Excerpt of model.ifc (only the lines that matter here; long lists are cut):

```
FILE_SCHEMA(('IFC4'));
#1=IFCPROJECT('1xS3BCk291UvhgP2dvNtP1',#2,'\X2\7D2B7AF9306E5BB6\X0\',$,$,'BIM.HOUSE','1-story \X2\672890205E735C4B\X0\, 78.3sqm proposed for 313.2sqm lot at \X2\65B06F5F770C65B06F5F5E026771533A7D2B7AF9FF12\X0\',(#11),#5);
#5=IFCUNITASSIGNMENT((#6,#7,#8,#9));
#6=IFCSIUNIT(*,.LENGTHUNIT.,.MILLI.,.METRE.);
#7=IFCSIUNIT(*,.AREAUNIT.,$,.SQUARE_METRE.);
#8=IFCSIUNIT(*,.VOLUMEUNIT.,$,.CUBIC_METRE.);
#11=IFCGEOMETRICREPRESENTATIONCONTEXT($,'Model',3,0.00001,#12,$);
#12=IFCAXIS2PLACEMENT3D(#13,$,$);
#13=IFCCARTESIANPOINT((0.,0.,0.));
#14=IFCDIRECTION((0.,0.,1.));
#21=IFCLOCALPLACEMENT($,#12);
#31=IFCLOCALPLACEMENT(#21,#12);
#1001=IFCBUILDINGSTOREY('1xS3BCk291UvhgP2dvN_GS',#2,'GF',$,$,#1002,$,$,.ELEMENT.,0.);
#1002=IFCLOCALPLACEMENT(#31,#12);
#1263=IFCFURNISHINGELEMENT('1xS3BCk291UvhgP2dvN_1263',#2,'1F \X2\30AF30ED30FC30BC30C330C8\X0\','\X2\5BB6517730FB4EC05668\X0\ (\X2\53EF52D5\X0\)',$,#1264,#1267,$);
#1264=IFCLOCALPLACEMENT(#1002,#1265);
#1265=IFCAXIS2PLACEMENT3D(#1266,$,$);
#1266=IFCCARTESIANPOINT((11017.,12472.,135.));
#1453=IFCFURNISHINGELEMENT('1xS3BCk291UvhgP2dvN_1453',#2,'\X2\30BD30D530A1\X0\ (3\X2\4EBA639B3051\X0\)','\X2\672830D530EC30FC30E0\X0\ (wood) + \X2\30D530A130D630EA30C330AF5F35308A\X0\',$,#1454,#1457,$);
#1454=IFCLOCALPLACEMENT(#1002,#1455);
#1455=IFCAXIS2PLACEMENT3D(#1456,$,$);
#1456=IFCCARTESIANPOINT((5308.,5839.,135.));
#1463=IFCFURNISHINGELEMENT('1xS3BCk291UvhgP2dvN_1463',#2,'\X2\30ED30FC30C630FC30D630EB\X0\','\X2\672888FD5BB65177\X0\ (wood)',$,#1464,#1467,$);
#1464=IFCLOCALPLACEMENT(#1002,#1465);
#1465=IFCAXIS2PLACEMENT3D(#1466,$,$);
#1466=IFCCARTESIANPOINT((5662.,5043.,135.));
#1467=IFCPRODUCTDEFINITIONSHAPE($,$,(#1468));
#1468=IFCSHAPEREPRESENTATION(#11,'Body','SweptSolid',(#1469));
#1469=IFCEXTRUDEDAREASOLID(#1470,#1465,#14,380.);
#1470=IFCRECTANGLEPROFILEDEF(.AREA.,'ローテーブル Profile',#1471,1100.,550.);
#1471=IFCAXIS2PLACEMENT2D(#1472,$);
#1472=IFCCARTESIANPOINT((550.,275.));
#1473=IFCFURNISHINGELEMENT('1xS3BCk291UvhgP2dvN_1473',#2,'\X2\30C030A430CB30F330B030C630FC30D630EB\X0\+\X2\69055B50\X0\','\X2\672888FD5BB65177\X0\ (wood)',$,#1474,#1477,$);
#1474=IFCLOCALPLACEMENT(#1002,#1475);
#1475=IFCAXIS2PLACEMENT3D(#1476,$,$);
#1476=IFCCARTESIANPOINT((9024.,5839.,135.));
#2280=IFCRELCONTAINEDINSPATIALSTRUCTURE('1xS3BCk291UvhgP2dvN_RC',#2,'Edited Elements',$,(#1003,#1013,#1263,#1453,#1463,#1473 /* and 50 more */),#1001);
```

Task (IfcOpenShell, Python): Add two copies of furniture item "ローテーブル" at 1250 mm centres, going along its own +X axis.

```python
import ifcopenshell
import ifcopenshell.api.geometry
import ifcopenshell.api.root
import ifcopenshell.util.element
import ifcopenshell.util.placement

model = ifcopenshell.open("model.ifc")


def reuse_history(source, copy):
    """copy_class also copies each property set's owner history, people and application; keep the originals."""
    for rel in copy.IsDefinedBy:
        if rel.is_a("IfcRelDefinesByProperties") and (history := rel.RelatingPropertyDefinition.OwnerHistory):
            rel.RelatingPropertyDefinition.OwnerHistory = source.OwnerHistory
            ifcopenshell.util.element.remove_deep2(model, history)


source = model.by_guid("1xS3BCk291UvhgP2dvN_1463")
base = ifcopenshell.util.placement.get_local_placement(source.ObjectPlacement)
step = base[:3, 0] * 1250.0

for i in range(1, 3):
    copy = ifcopenshell.api.root.copy_class(model, product=source)
    copy.Representation = ifcopenshell.util.element.copy_deep(
        model, source.Representation, exclude=["IfcGeometricRepresentationContext", "IfcRepresentationMap"]
    )
    reuse_history(source, copy)
    matrix = base.copy()
    matrix[:3, 3] += i * step
    print("added at", matrix[:3, 3].round(3) + 0.0)
    ifcopenshell.api.geometry.edit_object_placement(model, product=copy, matrix=matrix, is_si=False)

model.write("model_v2.ifc")
```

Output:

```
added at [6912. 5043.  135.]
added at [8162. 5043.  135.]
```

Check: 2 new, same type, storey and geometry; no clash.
